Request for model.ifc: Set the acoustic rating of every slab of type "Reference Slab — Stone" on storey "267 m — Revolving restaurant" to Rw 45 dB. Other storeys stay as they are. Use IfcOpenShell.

First a look at what the model holds.

```python
import ifcopenshell
import ifcopenshell.util.element

model = ifcopenshell.open("model.ifc")
print(model.schema)
storey = next(s for s in model.by_type("IfcBuildingStorey") if s.Name == "267 m — Revolving restaurant")
slabs = [e for e in ifcopenshell.util.element.get_decomposition(storey) if e.is_a("IfcSlab")]
seen = {}
for e in slabs:
    element_type = ifcopenshell.util.element.get_type(e)
    key = (element_type.Name if element_type != e and element_type else None, ifcopenshell.util.element.get_pset(e, "Pset_SlabCommon", "AcousticRating"))
    seen[key] = seen.get(key, 0) + 1
for (name, value), count in sorted(seen.items(), key=str):
    print(count, "x", name, "|", value)
```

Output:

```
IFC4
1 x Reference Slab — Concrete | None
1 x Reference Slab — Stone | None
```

```python
import ifcopenshell
import ifcopenshell.api.pset
import ifcopenshell.util.element

model = ifcopenshell.open("model.ifc")

storey = next(s for s in model.by_type("IfcBuildingStorey") if s.Name == "267 m — Revolving restaurant")
slabs = [e for e in ifcopenshell.util.element.get_decomposition(storey) if e.is_a("IfcSlab")]

count = 0
for e in slabs:
    element_type = ifcopenshell.util.element.get_type(e)
    if element_type in (None, e) or element_type.Name != "Reference Slab — Stone":
        continue
    # add_pset returns the element's existing set when there is one.
    pset = ifcopenshell.api.pset.add_pset(model, product=e, name="Pset_SlabCommon")
    ifcopenshell.api.pset.edit_pset(model, pset=pset, properties={"AcousticRating": "Rw 45 dB"})
    count += 1

print(count, "slabs updated")

model.write("model_updated.ifc")
```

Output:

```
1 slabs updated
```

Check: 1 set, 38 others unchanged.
